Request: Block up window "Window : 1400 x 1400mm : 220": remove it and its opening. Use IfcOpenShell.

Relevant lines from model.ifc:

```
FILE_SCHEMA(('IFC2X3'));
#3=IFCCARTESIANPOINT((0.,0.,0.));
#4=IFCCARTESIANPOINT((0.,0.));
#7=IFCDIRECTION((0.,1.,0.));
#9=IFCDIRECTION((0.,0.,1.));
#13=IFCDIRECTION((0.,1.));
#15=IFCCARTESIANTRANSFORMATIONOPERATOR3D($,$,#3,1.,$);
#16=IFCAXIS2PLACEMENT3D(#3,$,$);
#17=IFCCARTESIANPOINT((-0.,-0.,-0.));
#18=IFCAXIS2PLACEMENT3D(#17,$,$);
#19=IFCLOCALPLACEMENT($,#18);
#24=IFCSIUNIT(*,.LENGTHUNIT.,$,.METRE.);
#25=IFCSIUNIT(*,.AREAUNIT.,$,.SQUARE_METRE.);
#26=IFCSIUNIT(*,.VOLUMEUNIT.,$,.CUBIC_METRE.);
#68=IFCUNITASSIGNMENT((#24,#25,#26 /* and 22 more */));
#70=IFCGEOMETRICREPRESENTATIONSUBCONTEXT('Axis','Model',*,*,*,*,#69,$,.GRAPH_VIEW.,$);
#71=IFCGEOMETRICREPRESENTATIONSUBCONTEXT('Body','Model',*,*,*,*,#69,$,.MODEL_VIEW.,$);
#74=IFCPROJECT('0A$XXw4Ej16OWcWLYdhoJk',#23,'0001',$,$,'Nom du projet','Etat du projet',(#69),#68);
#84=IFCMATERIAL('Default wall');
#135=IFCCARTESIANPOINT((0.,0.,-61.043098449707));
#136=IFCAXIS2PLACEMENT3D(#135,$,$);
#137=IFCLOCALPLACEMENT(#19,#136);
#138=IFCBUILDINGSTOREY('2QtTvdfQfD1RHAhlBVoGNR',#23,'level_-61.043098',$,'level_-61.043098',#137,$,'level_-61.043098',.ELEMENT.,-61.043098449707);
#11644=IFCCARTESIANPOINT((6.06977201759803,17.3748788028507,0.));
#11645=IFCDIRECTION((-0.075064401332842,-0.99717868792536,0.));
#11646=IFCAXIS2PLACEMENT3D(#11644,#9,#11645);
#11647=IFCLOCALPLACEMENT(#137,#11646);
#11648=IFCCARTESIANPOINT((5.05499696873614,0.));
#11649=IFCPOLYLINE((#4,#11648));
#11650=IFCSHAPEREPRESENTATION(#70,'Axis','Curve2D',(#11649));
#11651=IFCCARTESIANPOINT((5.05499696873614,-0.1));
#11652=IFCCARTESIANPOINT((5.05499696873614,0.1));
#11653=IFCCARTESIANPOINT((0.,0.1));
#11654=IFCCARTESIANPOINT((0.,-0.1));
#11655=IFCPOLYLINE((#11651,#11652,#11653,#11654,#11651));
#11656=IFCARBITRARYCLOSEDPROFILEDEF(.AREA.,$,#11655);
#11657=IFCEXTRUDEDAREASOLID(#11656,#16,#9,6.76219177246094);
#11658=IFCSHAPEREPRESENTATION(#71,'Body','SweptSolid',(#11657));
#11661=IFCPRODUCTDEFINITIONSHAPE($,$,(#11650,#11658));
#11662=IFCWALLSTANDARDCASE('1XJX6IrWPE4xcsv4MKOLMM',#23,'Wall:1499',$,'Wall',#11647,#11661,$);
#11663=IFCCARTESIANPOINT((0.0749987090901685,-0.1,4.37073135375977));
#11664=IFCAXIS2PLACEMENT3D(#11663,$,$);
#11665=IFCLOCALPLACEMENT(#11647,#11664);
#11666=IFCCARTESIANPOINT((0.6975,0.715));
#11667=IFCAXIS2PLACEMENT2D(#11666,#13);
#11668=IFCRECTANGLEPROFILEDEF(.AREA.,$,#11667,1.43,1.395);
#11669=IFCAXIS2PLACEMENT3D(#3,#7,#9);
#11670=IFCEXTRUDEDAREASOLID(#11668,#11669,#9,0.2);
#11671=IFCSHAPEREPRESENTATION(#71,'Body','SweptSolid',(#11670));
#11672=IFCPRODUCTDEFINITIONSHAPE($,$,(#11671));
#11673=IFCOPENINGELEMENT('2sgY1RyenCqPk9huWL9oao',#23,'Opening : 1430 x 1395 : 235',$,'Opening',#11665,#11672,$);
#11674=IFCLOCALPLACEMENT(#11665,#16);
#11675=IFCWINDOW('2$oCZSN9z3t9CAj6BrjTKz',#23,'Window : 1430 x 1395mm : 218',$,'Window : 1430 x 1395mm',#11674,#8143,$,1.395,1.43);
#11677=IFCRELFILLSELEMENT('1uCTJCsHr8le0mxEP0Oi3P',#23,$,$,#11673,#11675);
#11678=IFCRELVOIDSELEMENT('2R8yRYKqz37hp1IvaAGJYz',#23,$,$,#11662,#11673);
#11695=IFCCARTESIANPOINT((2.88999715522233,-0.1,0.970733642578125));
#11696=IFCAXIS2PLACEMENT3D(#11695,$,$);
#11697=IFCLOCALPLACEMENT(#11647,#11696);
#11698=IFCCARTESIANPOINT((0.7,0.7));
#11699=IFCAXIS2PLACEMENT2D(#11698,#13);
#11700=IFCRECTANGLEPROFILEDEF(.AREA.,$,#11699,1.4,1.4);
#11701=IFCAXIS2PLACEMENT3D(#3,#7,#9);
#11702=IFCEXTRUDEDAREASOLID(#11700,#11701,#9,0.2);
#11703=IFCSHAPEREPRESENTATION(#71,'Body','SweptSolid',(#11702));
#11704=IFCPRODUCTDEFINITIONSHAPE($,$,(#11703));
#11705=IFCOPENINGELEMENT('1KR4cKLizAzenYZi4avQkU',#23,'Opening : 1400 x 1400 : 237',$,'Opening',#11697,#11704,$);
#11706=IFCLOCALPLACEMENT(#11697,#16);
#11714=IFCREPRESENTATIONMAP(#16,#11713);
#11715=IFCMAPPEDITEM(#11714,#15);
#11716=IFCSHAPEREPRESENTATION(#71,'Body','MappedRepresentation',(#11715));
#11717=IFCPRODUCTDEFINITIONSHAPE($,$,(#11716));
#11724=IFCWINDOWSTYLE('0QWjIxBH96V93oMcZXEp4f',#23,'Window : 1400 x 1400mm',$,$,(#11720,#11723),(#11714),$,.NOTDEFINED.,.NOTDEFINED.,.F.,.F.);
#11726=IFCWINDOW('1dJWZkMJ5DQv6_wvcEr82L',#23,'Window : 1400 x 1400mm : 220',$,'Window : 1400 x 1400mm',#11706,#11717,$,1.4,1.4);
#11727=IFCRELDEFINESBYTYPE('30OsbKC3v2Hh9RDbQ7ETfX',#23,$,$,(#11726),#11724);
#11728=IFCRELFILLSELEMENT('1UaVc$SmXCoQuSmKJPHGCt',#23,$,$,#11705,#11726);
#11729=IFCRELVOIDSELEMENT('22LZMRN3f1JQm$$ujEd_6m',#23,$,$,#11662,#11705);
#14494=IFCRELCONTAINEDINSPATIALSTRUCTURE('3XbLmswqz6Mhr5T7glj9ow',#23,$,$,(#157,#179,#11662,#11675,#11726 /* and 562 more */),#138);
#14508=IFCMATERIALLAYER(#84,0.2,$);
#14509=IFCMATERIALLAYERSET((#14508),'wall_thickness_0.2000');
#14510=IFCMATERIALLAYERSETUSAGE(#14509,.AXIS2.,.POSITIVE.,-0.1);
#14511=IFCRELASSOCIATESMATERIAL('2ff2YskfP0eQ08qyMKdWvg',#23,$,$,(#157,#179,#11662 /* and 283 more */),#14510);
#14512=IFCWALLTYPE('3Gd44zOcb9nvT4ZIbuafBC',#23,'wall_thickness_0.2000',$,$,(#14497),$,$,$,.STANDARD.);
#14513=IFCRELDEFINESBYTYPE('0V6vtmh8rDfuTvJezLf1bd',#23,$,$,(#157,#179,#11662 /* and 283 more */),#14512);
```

```python
import ifcopenshell
import ifcopenshell.api.feature
import ifcopenshell.api.root
import ifcopenshell.geom
import ifcopenshell.util.shape

model = ifcopenshell.open("model.ifc")
settings = ifcopenshell.geom.settings()


def volume(element):
    """Net volume in cubic metres, openings subtracted."""
    shape = ifcopenshell.geom.create_shape(settings, element)
    return ifcopenshell.util.shape.get_volume(shape.geometry)


window = model.by_guid("1dJWZkMJ5DQv6_wvcEr82L")
opening = window.FillsVoids[0].RelatingOpeningElement
wall = opening.VoidsElements[0].RelatingBuildingElement
before = volume(wall)

ifcopenshell.api.root.remove_product(model, product=window)
ifcopenshell.api.feature.remove_feature(model, feature=opening)

after = volume(wall)

print(f"wall volume {before:.3f} -> {after:.3f} m3")

model.write("model_edited.ifc")
```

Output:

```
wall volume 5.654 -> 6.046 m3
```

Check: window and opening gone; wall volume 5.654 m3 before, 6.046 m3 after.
